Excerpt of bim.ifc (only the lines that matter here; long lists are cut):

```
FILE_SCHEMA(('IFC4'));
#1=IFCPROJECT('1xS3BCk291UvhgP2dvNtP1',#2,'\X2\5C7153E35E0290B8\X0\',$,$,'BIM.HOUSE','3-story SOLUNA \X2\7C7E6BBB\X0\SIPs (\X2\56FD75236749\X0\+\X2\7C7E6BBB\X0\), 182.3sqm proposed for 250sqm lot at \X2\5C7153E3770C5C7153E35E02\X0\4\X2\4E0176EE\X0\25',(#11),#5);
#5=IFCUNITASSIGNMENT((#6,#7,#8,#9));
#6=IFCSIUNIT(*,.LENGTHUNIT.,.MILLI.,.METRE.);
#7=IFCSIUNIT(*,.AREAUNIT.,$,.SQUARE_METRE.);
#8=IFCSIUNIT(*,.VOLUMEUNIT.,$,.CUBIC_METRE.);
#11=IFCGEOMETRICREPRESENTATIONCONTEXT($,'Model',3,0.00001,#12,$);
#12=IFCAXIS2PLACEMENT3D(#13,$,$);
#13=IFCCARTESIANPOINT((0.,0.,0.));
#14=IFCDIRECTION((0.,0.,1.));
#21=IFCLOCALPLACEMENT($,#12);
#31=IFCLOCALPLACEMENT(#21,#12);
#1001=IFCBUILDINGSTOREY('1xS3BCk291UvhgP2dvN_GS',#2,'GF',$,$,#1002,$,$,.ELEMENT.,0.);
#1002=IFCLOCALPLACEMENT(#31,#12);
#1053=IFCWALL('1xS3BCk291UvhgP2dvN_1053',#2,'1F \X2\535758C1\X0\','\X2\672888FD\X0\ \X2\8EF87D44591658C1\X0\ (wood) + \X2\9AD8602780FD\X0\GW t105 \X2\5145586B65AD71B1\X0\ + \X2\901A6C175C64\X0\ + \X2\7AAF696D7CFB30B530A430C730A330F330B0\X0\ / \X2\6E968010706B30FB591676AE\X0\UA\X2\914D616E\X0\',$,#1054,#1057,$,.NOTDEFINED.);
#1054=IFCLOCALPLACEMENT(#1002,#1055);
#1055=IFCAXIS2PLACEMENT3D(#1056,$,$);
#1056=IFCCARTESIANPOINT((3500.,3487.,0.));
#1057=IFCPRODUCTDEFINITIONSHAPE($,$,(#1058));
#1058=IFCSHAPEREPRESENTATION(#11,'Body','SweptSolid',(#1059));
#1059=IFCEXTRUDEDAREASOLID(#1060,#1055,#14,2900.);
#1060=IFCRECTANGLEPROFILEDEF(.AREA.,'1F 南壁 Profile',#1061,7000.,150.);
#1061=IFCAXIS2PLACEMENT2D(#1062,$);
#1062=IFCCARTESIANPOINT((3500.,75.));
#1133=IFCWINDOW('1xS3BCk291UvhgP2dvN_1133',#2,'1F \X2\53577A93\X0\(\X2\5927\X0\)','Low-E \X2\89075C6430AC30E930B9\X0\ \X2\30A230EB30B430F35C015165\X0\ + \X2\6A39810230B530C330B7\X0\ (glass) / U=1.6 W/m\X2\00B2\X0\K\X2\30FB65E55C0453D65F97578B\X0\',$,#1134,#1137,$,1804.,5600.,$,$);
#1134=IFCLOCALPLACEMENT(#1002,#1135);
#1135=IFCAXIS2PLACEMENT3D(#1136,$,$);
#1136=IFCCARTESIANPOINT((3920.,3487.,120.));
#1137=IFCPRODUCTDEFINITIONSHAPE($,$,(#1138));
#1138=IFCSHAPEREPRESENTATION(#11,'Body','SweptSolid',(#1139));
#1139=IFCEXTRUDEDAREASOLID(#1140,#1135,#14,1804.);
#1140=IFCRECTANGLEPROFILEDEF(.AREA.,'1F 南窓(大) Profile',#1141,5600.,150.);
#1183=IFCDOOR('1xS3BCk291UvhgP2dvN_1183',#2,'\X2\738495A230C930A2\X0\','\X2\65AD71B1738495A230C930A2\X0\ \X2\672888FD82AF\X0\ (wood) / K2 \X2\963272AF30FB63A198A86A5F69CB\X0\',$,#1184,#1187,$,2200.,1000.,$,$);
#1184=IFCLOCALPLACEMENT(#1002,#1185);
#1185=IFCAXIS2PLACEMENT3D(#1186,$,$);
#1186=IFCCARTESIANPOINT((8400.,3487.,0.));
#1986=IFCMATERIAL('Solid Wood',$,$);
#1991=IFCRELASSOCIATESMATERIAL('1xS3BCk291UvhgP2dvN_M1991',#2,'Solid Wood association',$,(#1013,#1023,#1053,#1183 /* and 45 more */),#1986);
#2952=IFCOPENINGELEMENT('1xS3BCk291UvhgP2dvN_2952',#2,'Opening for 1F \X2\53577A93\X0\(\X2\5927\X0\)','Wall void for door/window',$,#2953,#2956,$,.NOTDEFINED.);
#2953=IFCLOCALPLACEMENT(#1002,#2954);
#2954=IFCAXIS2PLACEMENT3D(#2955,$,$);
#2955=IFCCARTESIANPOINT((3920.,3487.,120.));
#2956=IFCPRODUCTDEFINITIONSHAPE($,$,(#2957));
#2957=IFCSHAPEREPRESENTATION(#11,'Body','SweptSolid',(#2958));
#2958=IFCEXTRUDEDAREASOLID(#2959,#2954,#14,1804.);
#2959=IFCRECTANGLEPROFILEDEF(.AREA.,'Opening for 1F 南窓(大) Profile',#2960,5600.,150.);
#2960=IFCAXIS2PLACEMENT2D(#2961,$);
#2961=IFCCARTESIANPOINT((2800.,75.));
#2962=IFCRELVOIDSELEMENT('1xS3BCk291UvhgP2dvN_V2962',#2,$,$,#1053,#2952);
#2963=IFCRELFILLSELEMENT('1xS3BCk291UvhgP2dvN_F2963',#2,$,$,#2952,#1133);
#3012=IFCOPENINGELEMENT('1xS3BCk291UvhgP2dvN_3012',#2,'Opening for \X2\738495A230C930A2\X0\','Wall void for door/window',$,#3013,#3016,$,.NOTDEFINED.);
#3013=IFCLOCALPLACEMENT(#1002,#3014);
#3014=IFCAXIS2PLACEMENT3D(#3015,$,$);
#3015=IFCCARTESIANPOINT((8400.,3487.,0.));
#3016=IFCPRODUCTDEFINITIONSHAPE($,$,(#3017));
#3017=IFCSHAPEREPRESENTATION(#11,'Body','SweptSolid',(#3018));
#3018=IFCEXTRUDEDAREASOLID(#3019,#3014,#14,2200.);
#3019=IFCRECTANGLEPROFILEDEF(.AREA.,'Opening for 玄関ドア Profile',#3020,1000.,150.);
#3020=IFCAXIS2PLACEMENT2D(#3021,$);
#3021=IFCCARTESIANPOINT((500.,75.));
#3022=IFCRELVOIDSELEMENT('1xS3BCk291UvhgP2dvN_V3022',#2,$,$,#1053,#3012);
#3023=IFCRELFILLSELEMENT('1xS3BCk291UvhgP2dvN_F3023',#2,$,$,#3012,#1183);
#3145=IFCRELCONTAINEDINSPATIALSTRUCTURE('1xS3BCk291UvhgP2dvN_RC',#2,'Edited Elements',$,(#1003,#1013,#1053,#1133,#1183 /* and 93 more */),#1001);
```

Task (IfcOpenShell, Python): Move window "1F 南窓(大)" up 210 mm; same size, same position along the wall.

```python
import numpy as np
import ifcopenshell
import ifcopenshell.api.geometry
import ifcopenshell.util.placement
import ifcopenshell.util.unit

model = ifcopenshell.open("bim.ifc")
unit_scale = ifcopenshell.util.unit.calculate_unit_scale(model)

window = model.by_guid("1xS3BCk291UvhgP2dvN_1133")
opening = window.FillsVoids[0].RelatingOpeningElement
dz = 210.0

shift = np.array([0.0, 0.0, dz])
# The window is not placed relative to its opening, so move both.
for product in (opening, window):
    matrix = ifcopenshell.util.placement.get_local_placement(product.ObjectPlacement)
    matrix[:3, 3] += shift
    ifcopenshell.api.geometry.edit_object_placement(model, product=product, matrix=matrix, is_si=False)

print(f"moved by {dz * unit_scale:+.3f} m")

model.write("bim_updated.ifc")
```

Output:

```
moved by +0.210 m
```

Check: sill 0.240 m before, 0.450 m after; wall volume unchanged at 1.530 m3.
